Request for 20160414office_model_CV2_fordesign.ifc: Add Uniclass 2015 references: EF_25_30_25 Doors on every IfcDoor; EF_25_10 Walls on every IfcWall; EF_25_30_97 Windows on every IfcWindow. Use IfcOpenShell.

First a look at what the model holds.

```python
import ifcopenshell

model = ifcopenshell.open("20160414office_model_CV2_fordesign.ifc")
print(model.schema)
print("classifications:", [c.Name for c in model.by_type("IfcClassification")])
for ifc_class in ("IfcDoor", "IfcRoof", "IfcStair", "IfcWall", "IfcWindow"):
    print(ifc_class, len(model.by_type(ifc_class)))
```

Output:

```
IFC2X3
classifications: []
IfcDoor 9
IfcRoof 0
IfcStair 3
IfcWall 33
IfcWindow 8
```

```python
import ifcopenshell
import ifcopenshell.api.classification

model = ifcopenshell.open("20160414office_model_CV2_fordesign.ifc")

# IFC2X3 requires Source and Edition and has no link from the project to the system.
system = model.create_entity("IfcClassification", Source="NBS", Edition="2015", Name="Uniclass 2015")

codes = {
    "IfcDoor": ("EF_25_30_25", "Doors"),
    "IfcWall": ("EF_25_10", "Walls"),
    "IfcWindow": ("EF_25_30_97", "Windows"),
}
for ifc_class, (code, name) in codes.items():
    products = model.by_type(ifc_class)
    ifcopenshell.api.classification.add_reference(
        model, products=products, classification=system, identification=code, name=name
    )
    print(code, len(products))

model.write("20160414office_model_CV2_fordesign_edited.ifc")
```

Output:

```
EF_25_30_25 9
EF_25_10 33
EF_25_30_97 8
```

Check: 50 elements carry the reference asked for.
